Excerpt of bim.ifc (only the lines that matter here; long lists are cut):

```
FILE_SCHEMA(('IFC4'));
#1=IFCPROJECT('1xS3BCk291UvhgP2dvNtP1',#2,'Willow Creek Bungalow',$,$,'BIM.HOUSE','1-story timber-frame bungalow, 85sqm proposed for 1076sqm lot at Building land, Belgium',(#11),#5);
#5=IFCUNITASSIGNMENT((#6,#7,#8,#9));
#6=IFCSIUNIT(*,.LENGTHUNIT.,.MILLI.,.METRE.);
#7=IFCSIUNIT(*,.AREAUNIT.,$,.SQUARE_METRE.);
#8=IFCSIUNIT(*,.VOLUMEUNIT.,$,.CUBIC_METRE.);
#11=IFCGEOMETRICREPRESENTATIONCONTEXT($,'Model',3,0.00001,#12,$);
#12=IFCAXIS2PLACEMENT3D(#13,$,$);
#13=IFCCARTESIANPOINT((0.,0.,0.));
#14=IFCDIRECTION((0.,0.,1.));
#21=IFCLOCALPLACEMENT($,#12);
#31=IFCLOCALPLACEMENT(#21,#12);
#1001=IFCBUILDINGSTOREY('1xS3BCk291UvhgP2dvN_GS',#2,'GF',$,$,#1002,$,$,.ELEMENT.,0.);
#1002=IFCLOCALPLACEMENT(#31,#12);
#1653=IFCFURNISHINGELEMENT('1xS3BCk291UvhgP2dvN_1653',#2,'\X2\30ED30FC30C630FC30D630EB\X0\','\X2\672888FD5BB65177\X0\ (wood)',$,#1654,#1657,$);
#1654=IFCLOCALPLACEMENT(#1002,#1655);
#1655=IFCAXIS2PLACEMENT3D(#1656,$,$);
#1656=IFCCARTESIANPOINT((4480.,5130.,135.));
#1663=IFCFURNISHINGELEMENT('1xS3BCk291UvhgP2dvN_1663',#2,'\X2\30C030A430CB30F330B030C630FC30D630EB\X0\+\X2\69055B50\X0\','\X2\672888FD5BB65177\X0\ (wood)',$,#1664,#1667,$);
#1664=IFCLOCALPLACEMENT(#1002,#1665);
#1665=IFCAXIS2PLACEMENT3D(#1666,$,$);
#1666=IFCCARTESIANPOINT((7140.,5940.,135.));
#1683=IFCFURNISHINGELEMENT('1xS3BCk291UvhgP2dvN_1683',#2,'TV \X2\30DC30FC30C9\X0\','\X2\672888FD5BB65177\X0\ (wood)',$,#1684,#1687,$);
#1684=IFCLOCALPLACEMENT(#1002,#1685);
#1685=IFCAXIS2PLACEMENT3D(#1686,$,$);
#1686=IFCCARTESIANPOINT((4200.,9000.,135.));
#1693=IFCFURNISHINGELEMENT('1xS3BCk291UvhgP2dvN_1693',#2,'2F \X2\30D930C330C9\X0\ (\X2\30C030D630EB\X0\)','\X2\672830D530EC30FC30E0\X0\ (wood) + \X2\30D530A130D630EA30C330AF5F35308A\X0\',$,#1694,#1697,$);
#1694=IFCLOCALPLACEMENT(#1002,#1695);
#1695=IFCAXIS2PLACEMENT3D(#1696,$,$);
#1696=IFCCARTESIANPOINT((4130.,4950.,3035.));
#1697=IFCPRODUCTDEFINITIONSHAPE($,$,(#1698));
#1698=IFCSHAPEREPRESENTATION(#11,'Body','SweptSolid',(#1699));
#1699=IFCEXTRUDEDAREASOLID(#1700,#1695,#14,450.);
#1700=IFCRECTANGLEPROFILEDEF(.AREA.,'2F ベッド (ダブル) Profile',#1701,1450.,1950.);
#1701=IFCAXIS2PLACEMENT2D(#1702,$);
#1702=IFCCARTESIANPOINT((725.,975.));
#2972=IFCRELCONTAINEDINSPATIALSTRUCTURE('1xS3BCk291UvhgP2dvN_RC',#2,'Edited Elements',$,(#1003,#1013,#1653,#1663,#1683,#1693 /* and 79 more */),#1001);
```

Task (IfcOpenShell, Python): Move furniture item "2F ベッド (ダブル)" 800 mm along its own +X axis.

```python
import ifcopenshell
import ifcopenshell.api.geometry
import ifcopenshell.util.placement
import ifcopenshell.util.unit

model = ifcopenshell.open("bim.ifc")
unit_scale = ifcopenshell.util.unit.calculate_unit_scale(model)

item = model.by_id(1693)
matrix = ifcopenshell.util.placement.get_local_placement(item.ObjectPlacement)
matrix[:3, 3] += matrix[:3, 0] * 0.8 / unit_scale
ifcopenshell.api.geometry.edit_object_placement(model, product=item, matrix=matrix, is_si=False)

print(ifcopenshell.util.placement.get_local_placement(item.ObjectPlacement).round(3) + 0.0)

model.write("bim_edited.ifc")
```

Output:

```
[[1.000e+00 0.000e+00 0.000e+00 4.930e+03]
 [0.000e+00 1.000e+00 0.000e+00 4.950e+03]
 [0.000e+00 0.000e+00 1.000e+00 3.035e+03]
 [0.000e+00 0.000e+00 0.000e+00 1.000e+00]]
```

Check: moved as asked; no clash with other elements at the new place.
